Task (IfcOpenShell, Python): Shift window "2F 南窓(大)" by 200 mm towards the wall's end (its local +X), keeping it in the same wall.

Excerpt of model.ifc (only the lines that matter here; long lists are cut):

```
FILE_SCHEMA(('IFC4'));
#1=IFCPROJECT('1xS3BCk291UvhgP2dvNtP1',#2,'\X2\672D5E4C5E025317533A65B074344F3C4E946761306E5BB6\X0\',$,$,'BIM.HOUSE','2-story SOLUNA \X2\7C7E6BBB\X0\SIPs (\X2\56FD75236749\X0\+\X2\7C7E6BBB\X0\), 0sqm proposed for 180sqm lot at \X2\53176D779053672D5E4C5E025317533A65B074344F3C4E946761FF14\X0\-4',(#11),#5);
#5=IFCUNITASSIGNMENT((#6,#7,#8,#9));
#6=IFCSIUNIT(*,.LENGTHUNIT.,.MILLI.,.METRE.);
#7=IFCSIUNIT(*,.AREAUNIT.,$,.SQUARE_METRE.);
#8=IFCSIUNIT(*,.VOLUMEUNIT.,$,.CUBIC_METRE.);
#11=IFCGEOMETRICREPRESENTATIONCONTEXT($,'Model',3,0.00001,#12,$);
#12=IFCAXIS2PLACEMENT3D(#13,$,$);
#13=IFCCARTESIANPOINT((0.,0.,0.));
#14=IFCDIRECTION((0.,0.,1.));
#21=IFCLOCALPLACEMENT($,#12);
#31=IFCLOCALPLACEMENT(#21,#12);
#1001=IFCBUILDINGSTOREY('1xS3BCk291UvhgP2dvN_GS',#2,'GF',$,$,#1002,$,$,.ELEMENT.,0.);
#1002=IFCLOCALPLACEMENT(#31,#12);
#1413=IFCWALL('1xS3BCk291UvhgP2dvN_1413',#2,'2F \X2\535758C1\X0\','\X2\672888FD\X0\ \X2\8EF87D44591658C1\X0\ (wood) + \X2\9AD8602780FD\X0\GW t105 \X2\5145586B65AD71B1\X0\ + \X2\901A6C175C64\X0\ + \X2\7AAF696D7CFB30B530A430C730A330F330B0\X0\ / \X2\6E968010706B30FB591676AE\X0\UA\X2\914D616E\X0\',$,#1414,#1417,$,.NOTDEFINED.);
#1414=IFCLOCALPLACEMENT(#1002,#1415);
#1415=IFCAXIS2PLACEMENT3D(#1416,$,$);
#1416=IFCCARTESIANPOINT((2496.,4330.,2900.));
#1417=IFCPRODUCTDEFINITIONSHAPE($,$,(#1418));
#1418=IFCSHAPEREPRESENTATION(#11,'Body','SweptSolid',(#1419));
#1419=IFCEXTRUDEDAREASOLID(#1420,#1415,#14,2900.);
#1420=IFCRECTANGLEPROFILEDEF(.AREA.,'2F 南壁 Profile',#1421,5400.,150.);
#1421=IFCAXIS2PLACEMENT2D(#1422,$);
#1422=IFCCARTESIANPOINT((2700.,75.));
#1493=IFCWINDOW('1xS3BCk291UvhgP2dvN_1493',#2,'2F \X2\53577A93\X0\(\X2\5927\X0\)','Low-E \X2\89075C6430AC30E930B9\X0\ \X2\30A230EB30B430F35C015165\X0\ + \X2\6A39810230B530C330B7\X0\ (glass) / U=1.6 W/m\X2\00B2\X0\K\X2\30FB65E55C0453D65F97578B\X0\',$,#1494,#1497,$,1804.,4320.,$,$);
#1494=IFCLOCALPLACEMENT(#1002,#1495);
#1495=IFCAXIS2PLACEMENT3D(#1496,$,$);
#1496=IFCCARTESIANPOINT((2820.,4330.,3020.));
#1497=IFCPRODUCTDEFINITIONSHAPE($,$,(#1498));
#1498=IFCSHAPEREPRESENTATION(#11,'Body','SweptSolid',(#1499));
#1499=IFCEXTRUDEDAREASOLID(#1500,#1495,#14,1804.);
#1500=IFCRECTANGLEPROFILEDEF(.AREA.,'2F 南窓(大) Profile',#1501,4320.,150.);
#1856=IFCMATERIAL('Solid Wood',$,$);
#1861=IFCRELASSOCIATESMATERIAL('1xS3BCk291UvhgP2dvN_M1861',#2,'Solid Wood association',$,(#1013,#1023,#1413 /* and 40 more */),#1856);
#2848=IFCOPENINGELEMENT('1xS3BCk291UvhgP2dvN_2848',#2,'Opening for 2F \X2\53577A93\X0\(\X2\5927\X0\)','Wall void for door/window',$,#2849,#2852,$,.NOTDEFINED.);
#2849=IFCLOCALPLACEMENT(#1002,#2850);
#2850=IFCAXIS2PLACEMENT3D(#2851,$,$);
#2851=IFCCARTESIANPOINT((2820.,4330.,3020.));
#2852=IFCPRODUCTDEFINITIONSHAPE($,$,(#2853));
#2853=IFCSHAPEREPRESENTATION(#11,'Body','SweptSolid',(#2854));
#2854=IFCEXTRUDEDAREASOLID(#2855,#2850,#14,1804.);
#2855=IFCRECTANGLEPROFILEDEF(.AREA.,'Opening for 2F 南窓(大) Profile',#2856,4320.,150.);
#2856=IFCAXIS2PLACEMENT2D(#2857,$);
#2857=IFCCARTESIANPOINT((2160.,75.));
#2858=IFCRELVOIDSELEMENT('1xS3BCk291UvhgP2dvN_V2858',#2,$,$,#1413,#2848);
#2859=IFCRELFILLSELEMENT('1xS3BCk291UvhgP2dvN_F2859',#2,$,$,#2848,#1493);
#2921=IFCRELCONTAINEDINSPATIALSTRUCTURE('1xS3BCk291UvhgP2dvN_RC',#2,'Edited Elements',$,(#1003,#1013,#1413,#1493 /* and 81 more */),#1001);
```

```python
import ifcopenshell
import ifcopenshell.api.geometry
import ifcopenshell.util.placement

model = ifcopenshell.open("model.ifc")

window = model.by_id(1493)
opening = window.FillsVoids[0].RelatingOpeningElement
wall = opening.VoidsElements[0].RelatingBuildingElement

wall_matrix = ifcopenshell.util.placement.get_local_placement(wall.ObjectPlacement)
shift = wall_matrix[:3, 0] * 200.0
before = ifcopenshell.util.placement.get_local_placement(window.ObjectPlacement)[:3, 3].copy()

# The window is not placed relative to its opening, so move both.
for product in (opening, window):
    matrix = ifcopenshell.util.placement.get_local_placement(product.ObjectPlacement)
    matrix[:3, 3] += shift
    ifcopenshell.api.geometry.edit_object_placement(model, product=product, matrix=matrix, is_si=False)

after = ifcopenshell.util.placement.get_local_placement(window.ObjectPlacement)[:3, 3]
print("window moved by", (after - before).round(3) + 0.0)

model.write("model_updated.ifc")
```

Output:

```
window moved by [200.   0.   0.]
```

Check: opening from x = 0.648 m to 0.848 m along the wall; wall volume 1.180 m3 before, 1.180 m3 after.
